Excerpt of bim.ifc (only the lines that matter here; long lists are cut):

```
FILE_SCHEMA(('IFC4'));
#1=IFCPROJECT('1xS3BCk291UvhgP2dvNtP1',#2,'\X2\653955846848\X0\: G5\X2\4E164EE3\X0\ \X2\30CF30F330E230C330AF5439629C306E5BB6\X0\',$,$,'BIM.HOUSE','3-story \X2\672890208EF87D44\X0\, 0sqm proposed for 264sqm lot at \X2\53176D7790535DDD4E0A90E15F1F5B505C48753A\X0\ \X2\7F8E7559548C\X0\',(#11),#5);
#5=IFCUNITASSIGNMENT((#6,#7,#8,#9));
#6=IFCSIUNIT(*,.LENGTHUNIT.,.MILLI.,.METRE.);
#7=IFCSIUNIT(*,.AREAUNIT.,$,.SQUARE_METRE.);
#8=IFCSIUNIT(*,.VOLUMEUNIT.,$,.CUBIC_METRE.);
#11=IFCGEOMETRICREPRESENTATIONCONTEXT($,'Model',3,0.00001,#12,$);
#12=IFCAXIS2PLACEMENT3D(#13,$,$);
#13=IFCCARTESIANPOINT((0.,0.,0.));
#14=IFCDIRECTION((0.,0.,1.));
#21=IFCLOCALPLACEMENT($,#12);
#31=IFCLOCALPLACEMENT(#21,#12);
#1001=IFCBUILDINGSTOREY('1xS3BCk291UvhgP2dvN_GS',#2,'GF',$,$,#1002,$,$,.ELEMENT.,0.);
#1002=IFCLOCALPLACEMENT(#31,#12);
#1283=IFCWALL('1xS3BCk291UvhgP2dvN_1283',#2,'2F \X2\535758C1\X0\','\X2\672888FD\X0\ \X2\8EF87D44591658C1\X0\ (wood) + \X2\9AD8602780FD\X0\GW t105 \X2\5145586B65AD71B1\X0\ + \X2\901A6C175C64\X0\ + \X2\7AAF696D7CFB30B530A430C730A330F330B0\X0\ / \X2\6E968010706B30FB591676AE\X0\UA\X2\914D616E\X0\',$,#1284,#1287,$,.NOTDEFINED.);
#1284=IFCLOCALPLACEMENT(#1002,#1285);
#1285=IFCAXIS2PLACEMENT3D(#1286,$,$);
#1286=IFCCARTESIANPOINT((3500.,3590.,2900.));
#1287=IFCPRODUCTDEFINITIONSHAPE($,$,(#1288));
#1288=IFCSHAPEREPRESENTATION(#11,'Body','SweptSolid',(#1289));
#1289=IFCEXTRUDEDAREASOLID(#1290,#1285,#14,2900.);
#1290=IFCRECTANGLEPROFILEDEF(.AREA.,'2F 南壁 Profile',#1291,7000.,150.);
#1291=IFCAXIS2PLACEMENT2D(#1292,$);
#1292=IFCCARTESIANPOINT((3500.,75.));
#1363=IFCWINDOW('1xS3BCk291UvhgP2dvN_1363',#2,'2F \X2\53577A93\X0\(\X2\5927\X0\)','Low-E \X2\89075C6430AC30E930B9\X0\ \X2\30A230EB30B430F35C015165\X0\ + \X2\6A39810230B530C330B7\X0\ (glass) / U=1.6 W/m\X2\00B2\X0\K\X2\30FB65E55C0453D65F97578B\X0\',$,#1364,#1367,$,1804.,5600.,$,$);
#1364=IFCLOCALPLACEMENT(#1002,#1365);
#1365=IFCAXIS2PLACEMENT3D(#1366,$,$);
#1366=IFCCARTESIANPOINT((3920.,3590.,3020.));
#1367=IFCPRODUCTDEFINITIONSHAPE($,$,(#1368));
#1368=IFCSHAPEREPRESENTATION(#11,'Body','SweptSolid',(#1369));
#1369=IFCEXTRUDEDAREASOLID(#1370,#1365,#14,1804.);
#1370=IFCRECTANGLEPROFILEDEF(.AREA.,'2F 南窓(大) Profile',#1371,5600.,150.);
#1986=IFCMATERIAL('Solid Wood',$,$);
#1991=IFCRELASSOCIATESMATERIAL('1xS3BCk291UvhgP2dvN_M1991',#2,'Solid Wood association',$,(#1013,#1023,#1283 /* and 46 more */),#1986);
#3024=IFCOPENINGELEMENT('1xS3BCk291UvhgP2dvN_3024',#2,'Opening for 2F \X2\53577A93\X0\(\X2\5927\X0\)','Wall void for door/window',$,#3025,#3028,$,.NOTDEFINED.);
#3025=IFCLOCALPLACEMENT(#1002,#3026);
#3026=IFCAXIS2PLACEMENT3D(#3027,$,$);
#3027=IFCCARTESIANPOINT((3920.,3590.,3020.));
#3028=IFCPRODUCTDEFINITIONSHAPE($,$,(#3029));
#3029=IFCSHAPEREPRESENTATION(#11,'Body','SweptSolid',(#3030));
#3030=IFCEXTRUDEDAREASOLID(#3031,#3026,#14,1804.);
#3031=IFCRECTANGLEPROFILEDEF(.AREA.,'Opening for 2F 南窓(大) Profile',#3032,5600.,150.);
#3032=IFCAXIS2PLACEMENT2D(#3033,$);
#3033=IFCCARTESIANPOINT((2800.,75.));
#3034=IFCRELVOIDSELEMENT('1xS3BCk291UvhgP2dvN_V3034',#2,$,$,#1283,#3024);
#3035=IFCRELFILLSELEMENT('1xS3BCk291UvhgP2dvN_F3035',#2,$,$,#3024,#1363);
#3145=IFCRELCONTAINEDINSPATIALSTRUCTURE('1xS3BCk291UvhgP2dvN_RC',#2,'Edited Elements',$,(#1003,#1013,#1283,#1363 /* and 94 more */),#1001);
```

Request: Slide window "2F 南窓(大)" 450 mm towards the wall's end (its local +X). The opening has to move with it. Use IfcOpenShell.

```python
import ifcopenshell
import ifcopenshell.api.geometry
import ifcopenshell.util.placement
import ifcopenshell.util.unit

model = ifcopenshell.open("bim.ifc")
unit_scale = ifcopenshell.util.unit.calculate_unit_scale(model)

window = model.by_guid("1xS3BCk291UvhgP2dvN_1363")
opening = window.FillsVoids[0].RelatingOpeningElement
wall = opening.VoidsElements[0].RelatingBuildingElement

wall_matrix = ifcopenshell.util.placement.get_local_placement(wall.ObjectPlacement)
shift = wall_matrix[:3, 0] * 0.45 / unit_scale
before = ifcopenshell.util.placement.get_local_placement(window.ObjectPlacement)[:3, 3].copy()

# The window is not placed relative to its opening, so move both.
for product in (opening, window):
    matrix = ifcopenshell.util.placement.get_local_placement(product.ObjectPlacement)
    matrix[:3, 3] += shift
    ifcopenshell.api.geometry.edit_object_placement(model, product=product, matrix=matrix, is_si=False)

after = ifcopenshell.util.placement.get_local_placement(window.ObjectPlacement)[:3, 3]
print("window moved by", (after - before).round(3) + 0.0)

model.write("bim_rev.ifc")
```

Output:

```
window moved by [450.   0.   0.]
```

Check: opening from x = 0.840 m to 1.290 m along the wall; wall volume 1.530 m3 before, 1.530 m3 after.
